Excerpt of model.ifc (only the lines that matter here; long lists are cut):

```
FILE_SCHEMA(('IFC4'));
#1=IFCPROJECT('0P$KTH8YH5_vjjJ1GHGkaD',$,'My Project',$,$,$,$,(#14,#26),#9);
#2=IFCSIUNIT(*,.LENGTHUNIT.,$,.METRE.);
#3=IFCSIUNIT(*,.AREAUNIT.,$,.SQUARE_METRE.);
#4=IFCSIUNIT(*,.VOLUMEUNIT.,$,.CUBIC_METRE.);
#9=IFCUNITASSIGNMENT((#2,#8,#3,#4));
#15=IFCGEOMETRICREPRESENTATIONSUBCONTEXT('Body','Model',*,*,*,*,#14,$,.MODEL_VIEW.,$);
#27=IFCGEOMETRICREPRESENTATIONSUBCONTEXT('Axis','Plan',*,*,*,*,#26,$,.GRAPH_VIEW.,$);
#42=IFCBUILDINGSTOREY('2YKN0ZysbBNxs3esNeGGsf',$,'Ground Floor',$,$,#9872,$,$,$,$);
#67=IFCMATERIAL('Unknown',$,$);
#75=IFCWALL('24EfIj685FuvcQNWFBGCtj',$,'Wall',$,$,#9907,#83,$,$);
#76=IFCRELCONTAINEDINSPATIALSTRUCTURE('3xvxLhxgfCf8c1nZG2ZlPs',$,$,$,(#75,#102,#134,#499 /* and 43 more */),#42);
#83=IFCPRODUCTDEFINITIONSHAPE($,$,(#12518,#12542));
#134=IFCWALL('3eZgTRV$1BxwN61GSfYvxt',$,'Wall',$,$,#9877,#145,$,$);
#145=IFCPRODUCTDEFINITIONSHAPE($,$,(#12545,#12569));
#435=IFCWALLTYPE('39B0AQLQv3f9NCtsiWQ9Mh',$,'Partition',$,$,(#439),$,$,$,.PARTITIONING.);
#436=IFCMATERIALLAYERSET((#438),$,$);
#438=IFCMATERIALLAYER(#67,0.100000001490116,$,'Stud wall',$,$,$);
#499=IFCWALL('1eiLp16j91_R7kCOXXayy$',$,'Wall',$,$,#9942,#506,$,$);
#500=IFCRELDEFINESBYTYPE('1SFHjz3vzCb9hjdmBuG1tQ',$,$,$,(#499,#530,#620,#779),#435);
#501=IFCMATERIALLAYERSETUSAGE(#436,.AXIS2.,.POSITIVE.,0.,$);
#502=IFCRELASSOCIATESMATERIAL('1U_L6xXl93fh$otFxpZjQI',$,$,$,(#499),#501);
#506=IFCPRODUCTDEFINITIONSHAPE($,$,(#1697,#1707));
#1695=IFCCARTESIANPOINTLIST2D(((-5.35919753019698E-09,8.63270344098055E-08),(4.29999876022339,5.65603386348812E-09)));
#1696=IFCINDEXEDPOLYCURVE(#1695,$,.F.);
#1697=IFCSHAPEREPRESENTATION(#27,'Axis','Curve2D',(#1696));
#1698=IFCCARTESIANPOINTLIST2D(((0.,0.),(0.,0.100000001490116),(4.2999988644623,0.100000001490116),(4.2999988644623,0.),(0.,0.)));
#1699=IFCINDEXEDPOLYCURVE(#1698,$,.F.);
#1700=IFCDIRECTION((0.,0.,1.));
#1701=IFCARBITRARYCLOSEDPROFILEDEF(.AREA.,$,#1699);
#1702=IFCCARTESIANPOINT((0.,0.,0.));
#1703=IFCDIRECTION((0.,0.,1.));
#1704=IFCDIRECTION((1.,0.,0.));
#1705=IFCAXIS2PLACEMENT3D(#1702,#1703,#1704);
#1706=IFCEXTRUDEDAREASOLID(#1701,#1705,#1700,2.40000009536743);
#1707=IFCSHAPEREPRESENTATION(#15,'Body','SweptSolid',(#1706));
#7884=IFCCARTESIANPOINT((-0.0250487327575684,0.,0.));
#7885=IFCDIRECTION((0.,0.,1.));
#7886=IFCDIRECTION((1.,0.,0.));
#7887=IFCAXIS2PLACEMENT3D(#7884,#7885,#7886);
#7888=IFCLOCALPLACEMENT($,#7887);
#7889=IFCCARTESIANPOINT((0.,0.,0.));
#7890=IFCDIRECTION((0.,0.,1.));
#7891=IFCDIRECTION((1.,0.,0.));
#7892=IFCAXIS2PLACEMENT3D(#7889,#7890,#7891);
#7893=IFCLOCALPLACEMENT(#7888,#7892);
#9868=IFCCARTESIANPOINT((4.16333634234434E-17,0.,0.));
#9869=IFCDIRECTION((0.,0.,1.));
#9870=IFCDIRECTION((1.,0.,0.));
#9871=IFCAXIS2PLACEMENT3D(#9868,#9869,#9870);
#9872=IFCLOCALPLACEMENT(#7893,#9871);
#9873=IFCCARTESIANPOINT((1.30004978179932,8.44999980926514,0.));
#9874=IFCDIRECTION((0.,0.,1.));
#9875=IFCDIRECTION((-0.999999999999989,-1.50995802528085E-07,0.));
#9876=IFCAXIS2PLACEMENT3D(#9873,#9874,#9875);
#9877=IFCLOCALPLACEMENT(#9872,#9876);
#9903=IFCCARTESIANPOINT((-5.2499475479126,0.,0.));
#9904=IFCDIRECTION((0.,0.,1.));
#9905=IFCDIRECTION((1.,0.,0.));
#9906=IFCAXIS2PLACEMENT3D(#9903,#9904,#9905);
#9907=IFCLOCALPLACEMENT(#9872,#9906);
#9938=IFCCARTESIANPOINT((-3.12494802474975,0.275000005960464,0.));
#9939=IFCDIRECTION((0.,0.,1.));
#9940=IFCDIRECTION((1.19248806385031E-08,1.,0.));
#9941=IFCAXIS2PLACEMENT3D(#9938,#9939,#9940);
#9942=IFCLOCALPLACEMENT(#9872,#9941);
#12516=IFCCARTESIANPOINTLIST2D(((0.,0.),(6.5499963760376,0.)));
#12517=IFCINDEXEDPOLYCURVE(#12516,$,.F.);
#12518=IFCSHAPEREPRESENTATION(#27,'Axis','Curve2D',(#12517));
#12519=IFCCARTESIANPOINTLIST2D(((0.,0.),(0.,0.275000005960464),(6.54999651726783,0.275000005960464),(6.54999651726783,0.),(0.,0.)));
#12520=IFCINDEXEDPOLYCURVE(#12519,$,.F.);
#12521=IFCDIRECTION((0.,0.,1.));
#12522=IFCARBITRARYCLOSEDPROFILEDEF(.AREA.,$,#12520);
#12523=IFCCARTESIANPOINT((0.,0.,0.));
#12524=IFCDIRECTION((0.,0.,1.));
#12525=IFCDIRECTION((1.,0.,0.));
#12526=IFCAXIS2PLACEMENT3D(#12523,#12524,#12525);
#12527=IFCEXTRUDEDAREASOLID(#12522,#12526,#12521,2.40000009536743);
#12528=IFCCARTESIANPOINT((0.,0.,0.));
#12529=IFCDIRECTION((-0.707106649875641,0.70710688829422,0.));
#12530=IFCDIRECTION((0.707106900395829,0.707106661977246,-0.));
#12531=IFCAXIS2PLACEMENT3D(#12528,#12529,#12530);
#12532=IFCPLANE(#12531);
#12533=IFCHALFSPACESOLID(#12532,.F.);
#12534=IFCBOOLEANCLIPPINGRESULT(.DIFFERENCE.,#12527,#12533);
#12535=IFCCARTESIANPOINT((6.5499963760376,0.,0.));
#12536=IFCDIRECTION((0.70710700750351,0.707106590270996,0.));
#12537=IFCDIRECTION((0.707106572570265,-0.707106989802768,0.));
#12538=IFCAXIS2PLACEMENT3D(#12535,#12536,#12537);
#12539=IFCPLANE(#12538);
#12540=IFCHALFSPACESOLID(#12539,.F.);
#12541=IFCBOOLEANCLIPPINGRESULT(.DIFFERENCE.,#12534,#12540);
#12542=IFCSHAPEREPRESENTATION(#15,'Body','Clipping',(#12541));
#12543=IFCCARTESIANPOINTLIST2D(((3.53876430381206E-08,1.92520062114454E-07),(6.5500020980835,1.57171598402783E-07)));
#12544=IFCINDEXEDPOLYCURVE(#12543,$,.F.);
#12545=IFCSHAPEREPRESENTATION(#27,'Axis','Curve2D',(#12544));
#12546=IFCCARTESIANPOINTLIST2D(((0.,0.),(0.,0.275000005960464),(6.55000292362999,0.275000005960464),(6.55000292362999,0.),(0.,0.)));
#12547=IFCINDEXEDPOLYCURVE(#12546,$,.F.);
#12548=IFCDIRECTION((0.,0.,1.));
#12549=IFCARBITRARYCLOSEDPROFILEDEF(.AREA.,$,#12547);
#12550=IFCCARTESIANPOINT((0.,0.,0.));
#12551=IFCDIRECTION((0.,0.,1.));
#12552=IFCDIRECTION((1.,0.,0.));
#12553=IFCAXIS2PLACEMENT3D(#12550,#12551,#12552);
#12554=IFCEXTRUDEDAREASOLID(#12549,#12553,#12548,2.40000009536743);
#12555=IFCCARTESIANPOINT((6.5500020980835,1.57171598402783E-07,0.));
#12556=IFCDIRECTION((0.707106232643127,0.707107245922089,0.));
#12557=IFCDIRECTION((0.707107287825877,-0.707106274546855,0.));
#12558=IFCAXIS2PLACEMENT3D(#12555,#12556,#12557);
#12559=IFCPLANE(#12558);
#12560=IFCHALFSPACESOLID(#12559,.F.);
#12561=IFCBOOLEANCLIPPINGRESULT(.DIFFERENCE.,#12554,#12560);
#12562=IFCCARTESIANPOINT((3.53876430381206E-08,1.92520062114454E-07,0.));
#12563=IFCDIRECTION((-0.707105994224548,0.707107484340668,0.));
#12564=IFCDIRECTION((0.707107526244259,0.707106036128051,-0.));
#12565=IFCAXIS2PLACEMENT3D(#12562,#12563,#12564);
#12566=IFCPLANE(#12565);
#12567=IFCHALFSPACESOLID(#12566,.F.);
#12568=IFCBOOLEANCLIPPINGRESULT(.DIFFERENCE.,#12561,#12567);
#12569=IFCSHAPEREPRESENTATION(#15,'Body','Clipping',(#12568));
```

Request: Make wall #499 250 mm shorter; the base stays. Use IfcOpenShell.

```python
import ifcopenshell
import ifcopenshell.geom
import ifcopenshell.util.representation
import ifcopenshell.util.shape

model = ifcopenshell.open("model.ifc")
settings = ifcopenshell.geom.settings()


def volume(element):
    """Net volume in cubic metres, openings subtracted."""
    shape = ifcopenshell.geom.create_shape(settings, element)
    return ifcopenshell.util.shape.get_volume(shape.geometry)


wall = model.by_guid("1eiLp16j91_R7kCOXXayy$")
before = volume(wall)

body = ifcopenshell.util.representation.get_representation(wall, "Model", "Body")
solid = body.Items[0]
old_height = solid.Depth
solid.Depth -= 0.25
after = volume(wall)

print(f"height {old_height:g} -> {solid.Depth:g}, volume {before:.3f} -> {after:.3f} m3")

model.write("model-out.ifc")
```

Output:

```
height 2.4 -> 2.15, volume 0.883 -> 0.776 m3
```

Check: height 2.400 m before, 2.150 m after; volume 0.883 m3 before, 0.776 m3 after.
